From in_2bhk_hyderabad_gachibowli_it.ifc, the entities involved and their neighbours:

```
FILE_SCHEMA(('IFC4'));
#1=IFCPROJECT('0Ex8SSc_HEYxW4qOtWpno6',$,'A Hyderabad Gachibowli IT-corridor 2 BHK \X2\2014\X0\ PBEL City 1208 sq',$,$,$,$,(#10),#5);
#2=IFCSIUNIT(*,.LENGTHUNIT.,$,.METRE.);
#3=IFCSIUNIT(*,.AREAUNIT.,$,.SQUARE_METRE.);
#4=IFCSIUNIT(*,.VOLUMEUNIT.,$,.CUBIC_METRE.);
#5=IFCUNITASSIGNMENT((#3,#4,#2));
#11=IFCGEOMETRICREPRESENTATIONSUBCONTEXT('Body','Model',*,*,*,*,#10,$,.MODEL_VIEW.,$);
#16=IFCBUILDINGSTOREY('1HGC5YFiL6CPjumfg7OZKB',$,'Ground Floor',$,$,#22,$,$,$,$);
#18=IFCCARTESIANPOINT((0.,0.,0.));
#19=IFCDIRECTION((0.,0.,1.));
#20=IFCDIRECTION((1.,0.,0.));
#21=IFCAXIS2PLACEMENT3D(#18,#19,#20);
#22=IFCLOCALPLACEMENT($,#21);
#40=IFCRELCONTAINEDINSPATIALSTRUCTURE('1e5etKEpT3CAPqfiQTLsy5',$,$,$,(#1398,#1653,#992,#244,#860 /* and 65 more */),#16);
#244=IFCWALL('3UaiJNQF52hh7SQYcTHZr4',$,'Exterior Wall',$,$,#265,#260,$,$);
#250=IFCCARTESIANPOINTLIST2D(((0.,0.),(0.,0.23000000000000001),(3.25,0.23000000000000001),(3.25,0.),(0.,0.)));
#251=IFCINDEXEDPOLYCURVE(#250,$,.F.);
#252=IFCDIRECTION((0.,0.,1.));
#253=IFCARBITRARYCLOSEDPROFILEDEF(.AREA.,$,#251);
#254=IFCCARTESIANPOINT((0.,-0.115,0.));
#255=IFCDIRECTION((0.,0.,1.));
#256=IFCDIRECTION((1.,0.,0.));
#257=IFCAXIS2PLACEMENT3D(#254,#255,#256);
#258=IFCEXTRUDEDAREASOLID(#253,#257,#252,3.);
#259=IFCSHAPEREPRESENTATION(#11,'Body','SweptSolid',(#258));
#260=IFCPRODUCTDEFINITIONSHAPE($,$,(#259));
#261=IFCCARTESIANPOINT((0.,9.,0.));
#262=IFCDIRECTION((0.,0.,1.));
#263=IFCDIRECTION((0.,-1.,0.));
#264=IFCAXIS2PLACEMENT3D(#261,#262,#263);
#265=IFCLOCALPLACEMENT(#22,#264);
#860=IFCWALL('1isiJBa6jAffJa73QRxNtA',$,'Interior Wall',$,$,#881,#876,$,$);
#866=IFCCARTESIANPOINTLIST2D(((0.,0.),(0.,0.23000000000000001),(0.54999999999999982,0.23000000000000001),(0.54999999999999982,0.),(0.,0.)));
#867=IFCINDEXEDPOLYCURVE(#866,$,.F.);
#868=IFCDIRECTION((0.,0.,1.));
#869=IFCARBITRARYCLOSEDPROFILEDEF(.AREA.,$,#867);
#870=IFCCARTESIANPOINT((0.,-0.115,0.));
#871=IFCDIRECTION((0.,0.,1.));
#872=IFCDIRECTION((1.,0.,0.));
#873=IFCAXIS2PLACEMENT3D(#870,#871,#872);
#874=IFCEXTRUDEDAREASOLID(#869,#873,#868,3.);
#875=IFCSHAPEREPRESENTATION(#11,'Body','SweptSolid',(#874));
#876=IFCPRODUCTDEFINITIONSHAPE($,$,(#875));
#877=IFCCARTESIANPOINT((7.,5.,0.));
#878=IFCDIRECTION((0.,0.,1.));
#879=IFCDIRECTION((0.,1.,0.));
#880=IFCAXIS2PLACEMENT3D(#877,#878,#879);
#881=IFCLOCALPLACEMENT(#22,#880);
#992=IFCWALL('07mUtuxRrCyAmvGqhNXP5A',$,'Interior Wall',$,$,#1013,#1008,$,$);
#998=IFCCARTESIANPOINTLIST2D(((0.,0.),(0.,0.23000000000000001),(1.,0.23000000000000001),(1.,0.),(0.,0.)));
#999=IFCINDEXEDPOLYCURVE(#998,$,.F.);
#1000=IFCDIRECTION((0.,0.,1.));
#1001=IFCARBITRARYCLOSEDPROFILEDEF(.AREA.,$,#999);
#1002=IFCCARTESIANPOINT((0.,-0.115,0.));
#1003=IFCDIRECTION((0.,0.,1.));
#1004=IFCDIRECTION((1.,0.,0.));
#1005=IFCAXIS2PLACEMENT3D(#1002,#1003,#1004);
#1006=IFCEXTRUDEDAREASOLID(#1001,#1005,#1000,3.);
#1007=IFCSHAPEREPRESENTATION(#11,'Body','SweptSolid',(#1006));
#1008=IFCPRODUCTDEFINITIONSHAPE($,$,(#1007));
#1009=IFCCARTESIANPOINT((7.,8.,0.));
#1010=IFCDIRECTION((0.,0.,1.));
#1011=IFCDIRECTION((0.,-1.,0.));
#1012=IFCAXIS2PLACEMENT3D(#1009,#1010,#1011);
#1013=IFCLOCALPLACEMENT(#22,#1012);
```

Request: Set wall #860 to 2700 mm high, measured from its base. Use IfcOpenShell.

```python
import ifcopenshell
import ifcopenshell.geom
import ifcopenshell.util.representation
import ifcopenshell.util.shape

model = ifcopenshell.open("in_2bhk_hyderabad_gachibowli_it.ifc")
settings = ifcopenshell.geom.settings()


def volume(element):
    """Net volume in cubic metres, openings subtracted."""
    shape = ifcopenshell.geom.create_shape(settings, element)
    return ifcopenshell.util.shape.get_volume(shape.geometry)


wall = model.by_id(860)
before = volume(wall)

body = ifcopenshell.util.representation.get_representation(wall, "Model", "Body")
solid = body.Items[0]
old_height = solid.Depth
solid.Depth = 2.7
after = volume(wall)

print(f"height {old_height:g} -> {solid.Depth:g}, volume {before:.3f} -> {after:.3f} m3")

model.write("in_2bhk_hyderabad_gachibowli_it_v2.ifc")
```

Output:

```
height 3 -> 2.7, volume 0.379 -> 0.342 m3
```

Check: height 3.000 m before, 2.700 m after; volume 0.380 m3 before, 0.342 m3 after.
